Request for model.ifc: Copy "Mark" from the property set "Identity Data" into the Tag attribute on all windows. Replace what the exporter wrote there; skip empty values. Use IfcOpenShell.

First a look at what the model holds.

```python
import ifcopenshell
import ifcopenshell.util.element

model = ifcopenshell.open("model.ifc")
print(model.schema)
windows = model.by_type("IfcWindow")
print(len(windows), "windows")
for e in windows[:8]:
    source = ifcopenshell.util.element.get_pset(e, "Identity Data", "Mark")
    target = e.Tag
    print(e.id(), repr(source), repr(target), sep=" | ")
```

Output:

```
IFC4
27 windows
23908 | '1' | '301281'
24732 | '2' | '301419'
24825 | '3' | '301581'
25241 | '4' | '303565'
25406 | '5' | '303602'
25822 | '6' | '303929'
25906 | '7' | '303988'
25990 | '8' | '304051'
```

```python
import ifcopenshell
import ifcopenshell.util.element

model = ifcopenshell.open("model.ifc")

count = 0
for e in model.by_type("IfcWindow"):
    value = ifcopenshell.util.element.get_pset(e, "Identity Data", "Mark")
    current = e.Tag
    if not value or not value.strip() or current == value:
        continue
    e.Tag = value
    count += 1

print(count, "windows updated")

model.write("model_v2.ifc")
```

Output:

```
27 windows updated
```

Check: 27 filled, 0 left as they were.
